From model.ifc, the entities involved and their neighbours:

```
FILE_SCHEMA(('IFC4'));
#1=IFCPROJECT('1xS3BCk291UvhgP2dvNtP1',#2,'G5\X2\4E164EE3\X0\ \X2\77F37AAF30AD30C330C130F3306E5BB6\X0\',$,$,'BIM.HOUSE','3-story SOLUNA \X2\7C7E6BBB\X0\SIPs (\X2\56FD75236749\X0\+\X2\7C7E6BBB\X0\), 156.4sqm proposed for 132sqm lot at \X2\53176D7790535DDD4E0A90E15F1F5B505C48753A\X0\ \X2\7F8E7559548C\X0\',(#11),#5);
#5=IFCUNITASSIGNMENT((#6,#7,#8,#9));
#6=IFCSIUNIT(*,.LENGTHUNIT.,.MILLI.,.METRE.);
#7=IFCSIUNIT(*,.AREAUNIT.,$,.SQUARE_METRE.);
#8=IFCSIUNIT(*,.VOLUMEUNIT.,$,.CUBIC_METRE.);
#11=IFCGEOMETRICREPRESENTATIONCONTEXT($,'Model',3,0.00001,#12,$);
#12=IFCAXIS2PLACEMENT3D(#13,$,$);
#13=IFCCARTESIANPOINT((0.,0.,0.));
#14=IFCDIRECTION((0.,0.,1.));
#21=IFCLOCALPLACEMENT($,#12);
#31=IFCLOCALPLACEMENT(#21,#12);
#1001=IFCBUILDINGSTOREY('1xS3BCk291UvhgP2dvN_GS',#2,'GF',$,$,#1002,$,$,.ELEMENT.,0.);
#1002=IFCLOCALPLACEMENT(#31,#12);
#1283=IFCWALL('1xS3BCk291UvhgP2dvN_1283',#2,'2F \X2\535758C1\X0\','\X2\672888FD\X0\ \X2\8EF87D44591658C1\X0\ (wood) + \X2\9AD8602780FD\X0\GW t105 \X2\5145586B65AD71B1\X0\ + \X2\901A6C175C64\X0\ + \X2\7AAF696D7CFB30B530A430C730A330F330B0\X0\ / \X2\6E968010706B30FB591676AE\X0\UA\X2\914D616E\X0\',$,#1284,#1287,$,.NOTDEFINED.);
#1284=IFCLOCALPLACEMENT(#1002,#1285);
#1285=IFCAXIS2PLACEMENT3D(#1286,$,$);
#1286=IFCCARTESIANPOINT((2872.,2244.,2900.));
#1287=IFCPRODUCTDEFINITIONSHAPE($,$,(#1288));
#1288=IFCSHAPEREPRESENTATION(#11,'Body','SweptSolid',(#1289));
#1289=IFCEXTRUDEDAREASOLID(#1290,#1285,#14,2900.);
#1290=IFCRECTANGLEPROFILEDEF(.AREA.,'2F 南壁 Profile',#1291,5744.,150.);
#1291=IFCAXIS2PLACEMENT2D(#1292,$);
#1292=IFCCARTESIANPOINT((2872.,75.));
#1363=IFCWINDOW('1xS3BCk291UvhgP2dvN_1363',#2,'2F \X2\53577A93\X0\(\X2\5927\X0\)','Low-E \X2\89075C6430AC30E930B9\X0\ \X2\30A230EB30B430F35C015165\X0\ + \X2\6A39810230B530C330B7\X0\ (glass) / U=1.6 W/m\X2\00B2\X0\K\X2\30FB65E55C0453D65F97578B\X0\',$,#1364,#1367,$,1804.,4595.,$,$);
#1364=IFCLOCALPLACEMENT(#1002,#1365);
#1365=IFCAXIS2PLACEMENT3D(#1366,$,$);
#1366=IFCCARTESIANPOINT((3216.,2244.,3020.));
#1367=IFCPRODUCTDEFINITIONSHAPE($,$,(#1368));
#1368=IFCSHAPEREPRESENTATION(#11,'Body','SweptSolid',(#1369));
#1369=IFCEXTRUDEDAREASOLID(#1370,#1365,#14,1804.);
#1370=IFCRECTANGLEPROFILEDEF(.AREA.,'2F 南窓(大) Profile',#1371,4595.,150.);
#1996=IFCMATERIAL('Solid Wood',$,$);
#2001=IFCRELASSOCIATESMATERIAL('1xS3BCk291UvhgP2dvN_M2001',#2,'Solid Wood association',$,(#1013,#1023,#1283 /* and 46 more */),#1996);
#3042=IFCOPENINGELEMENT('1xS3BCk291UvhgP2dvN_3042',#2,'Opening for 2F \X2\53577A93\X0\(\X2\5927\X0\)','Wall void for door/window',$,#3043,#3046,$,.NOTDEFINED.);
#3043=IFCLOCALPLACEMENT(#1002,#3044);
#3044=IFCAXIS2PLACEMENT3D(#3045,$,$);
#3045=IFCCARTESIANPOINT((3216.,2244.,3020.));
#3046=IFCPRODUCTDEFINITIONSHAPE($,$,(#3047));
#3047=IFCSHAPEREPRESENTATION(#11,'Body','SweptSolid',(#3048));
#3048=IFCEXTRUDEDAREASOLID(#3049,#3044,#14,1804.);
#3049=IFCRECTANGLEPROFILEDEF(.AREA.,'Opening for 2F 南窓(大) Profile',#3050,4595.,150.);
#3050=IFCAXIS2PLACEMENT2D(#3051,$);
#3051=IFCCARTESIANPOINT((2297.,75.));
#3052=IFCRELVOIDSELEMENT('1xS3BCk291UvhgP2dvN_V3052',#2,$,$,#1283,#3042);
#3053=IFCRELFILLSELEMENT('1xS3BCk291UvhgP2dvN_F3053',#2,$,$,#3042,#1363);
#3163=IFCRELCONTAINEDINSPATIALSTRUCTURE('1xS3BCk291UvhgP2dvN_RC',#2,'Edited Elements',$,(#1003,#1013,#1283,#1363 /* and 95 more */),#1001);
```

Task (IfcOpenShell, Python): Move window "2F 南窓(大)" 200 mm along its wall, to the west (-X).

```python
import ifcopenshell
import ifcopenshell.api.geometry
import ifcopenshell.util.placement
import ifcopenshell.util.unit

model = ifcopenshell.open("model.ifc")
unit_scale = ifcopenshell.util.unit.calculate_unit_scale(model)

window = model.by_id(1363)
opening = window.FillsVoids[0].RelatingOpeningElement
wall = opening.VoidsElements[0].RelatingBuildingElement

wall_matrix = ifcopenshell.util.placement.get_local_placement(wall.ObjectPlacement)
shift = wall_matrix[:3, 0] * -0.2 / unit_scale
before = ifcopenshell.util.placement.get_local_placement(window.ObjectPlacement)[:3, 3].copy()

# The window is not placed relative to its opening, so move both.
for product in (opening, window):
    matrix = ifcopenshell.util.placement.get_local_placement(product.ObjectPlacement)
    matrix[:3, 3] += shift
    ifcopenshell.api.geometry.edit_object_placement(model, product=product, matrix=matrix, is_si=False)

after = ifcopenshell.util.placement.get_local_placement(window.ObjectPlacement)[:3, 3]
print("window moved by", (after - before).round(3) + 0.0)

model.write("model_edited.ifc")
```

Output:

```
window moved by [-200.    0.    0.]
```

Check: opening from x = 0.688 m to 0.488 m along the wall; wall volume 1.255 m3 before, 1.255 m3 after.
